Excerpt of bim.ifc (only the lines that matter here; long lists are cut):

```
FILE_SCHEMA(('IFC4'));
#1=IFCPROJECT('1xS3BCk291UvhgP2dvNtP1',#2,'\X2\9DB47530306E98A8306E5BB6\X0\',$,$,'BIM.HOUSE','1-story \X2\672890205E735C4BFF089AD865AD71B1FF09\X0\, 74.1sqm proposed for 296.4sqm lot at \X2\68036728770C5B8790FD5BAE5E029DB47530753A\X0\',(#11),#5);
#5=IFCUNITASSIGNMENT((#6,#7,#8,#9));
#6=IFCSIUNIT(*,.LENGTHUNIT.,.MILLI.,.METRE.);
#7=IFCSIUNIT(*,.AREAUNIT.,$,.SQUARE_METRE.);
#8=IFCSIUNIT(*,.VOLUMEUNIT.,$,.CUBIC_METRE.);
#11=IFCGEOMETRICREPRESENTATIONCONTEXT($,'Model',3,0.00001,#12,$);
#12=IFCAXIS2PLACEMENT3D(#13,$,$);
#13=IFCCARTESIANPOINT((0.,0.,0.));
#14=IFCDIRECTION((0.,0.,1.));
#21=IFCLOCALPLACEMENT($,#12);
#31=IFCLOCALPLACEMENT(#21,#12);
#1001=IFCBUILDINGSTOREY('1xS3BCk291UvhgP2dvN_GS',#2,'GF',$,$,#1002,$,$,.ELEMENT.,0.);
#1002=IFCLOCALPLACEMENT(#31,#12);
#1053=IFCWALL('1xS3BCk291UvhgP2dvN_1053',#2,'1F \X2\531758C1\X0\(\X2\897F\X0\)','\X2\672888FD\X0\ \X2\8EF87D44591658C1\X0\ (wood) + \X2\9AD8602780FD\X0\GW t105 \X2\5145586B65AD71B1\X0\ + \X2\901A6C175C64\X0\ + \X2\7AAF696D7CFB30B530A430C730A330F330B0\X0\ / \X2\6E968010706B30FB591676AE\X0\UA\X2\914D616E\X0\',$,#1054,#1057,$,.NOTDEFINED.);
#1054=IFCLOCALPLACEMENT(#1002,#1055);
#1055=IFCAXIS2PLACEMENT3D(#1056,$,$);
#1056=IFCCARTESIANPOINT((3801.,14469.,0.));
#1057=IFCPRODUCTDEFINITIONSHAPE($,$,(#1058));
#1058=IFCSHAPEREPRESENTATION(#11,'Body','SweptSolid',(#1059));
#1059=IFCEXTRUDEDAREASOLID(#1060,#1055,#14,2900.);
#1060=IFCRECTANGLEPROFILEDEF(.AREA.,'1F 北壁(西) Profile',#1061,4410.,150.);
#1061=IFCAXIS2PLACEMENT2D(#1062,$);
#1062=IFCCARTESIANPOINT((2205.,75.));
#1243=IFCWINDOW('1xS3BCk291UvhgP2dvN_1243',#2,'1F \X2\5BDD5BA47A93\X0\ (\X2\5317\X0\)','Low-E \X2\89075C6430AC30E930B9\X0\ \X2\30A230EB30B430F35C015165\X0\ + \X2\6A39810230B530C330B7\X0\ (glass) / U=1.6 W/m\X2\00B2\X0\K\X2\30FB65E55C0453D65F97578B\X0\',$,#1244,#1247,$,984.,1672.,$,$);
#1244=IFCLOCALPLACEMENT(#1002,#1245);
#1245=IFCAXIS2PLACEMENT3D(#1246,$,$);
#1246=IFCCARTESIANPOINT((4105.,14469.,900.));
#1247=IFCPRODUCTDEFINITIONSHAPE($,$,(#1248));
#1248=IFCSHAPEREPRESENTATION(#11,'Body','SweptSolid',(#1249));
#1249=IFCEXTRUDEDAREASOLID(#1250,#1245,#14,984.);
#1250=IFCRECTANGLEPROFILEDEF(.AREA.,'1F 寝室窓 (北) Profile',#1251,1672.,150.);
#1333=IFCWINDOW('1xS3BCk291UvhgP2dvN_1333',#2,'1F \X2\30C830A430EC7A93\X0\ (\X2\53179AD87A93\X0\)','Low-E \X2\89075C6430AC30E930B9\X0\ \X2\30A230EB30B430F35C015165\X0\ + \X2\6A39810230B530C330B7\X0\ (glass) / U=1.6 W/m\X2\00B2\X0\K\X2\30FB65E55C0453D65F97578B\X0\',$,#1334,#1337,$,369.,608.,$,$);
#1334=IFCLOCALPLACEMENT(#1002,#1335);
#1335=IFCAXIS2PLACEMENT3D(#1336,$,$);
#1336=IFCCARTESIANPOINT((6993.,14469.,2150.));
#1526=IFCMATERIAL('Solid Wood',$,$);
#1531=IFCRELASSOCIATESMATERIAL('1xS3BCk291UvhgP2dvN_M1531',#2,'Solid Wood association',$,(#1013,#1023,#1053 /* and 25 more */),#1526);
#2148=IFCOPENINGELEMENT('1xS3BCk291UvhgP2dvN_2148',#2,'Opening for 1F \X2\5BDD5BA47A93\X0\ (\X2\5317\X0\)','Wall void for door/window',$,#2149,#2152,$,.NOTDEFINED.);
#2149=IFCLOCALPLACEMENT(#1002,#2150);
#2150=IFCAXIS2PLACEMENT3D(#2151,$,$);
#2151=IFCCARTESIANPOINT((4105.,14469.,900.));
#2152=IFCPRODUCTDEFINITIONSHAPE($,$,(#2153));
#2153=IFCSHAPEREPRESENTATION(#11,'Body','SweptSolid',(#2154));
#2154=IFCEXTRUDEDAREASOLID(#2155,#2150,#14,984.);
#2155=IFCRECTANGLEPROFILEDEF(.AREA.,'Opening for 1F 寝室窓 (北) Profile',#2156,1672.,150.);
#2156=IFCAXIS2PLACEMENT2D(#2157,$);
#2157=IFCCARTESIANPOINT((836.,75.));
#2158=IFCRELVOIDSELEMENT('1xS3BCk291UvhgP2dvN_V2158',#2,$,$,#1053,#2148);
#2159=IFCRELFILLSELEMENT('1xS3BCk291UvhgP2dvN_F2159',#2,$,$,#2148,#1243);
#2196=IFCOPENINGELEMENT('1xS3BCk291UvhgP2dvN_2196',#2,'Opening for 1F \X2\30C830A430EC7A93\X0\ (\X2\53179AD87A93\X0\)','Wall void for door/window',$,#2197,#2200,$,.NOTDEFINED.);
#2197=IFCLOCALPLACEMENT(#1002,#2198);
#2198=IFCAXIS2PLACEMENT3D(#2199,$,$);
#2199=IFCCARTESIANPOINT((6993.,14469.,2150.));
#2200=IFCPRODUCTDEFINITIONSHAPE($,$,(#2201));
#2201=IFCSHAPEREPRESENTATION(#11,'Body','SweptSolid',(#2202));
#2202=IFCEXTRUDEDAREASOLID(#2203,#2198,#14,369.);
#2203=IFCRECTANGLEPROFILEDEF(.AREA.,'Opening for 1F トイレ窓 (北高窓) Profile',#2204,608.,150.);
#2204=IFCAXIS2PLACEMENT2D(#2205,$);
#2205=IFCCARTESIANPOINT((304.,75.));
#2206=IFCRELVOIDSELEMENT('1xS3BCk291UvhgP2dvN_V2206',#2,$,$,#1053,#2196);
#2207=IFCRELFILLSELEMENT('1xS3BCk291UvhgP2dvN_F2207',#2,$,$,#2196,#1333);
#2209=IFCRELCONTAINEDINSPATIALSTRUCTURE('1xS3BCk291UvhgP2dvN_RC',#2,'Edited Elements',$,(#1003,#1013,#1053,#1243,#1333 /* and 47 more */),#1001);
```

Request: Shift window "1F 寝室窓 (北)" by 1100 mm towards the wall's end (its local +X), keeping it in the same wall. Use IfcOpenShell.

```python
import ifcopenshell
import ifcopenshell.api.geometry
import ifcopenshell.util.placement
import ifcopenshell.util.unit

model = ifcopenshell.open("bim.ifc")
unit_scale = ifcopenshell.util.unit.calculate_unit_scale(model)

window = model.by_guid("1xS3BCk291UvhgP2dvN_1243")
opening = window.FillsVoids[0].RelatingOpeningElement
wall = opening.VoidsElements[0].RelatingBuildingElement

wall_matrix = ifcopenshell.util.placement.get_local_placement(wall.ObjectPlacement)
shift = wall_matrix[:3, 0] * 1.1 / unit_scale
before = ifcopenshell.util.placement.get_local_placement(window.ObjectPlacement)[:3, 3].copy()

# The window is not placed relative to its opening, so move both.
for product in (opening, window):
    matrix = ifcopenshell.util.placement.get_local_placement(product.ObjectPlacement)
    matrix[:3, 3] += shift
    ifcopenshell.api.geometry.edit_object_placement(model, product=product, matrix=matrix, is_si=False)

after = ifcopenshell.util.placement.get_local_placement(window.ObjectPlacement)[:3, 3]
print("window moved by", (after - before).round(3) + 0.0)

model.write("bim_v2.ifc")
```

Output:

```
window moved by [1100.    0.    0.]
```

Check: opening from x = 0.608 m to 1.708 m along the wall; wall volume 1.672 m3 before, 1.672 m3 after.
